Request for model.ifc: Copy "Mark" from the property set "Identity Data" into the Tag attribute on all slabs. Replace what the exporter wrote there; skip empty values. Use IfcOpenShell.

First a look at what the model holds.

```python
import ifcopenshell
import ifcopenshell.util.element

model = ifcopenshell.open("model.ifc")
print(model.schema)
slabs = model.by_type("IfcSlab")
print(len(slabs), "slabs")
for e in slabs[:8]:
    source = ifcopenshell.util.element.get_pset(e, "Identity Data", "Mark")
    target = e.Tag
    print(e.id(), repr(source), repr(target), sep=" | ")
```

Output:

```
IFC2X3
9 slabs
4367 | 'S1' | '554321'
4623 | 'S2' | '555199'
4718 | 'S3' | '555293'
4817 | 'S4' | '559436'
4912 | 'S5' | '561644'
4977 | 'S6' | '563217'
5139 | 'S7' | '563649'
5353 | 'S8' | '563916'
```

```python
import ifcopenshell
import ifcopenshell.util.element

model = ifcopenshell.open("model.ifc")

count = 0
for e in model.by_type("IfcSlab"):
    value = ifcopenshell.util.element.get_pset(e, "Identity Data", "Mark")
    current = e.Tag
    if not value or not value.strip() or current == value:
        continue
    e.Tag = value
    count += 1

print(count, "slabs updated")

model.write("model_rev.ifc")
```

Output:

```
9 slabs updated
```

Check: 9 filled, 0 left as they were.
